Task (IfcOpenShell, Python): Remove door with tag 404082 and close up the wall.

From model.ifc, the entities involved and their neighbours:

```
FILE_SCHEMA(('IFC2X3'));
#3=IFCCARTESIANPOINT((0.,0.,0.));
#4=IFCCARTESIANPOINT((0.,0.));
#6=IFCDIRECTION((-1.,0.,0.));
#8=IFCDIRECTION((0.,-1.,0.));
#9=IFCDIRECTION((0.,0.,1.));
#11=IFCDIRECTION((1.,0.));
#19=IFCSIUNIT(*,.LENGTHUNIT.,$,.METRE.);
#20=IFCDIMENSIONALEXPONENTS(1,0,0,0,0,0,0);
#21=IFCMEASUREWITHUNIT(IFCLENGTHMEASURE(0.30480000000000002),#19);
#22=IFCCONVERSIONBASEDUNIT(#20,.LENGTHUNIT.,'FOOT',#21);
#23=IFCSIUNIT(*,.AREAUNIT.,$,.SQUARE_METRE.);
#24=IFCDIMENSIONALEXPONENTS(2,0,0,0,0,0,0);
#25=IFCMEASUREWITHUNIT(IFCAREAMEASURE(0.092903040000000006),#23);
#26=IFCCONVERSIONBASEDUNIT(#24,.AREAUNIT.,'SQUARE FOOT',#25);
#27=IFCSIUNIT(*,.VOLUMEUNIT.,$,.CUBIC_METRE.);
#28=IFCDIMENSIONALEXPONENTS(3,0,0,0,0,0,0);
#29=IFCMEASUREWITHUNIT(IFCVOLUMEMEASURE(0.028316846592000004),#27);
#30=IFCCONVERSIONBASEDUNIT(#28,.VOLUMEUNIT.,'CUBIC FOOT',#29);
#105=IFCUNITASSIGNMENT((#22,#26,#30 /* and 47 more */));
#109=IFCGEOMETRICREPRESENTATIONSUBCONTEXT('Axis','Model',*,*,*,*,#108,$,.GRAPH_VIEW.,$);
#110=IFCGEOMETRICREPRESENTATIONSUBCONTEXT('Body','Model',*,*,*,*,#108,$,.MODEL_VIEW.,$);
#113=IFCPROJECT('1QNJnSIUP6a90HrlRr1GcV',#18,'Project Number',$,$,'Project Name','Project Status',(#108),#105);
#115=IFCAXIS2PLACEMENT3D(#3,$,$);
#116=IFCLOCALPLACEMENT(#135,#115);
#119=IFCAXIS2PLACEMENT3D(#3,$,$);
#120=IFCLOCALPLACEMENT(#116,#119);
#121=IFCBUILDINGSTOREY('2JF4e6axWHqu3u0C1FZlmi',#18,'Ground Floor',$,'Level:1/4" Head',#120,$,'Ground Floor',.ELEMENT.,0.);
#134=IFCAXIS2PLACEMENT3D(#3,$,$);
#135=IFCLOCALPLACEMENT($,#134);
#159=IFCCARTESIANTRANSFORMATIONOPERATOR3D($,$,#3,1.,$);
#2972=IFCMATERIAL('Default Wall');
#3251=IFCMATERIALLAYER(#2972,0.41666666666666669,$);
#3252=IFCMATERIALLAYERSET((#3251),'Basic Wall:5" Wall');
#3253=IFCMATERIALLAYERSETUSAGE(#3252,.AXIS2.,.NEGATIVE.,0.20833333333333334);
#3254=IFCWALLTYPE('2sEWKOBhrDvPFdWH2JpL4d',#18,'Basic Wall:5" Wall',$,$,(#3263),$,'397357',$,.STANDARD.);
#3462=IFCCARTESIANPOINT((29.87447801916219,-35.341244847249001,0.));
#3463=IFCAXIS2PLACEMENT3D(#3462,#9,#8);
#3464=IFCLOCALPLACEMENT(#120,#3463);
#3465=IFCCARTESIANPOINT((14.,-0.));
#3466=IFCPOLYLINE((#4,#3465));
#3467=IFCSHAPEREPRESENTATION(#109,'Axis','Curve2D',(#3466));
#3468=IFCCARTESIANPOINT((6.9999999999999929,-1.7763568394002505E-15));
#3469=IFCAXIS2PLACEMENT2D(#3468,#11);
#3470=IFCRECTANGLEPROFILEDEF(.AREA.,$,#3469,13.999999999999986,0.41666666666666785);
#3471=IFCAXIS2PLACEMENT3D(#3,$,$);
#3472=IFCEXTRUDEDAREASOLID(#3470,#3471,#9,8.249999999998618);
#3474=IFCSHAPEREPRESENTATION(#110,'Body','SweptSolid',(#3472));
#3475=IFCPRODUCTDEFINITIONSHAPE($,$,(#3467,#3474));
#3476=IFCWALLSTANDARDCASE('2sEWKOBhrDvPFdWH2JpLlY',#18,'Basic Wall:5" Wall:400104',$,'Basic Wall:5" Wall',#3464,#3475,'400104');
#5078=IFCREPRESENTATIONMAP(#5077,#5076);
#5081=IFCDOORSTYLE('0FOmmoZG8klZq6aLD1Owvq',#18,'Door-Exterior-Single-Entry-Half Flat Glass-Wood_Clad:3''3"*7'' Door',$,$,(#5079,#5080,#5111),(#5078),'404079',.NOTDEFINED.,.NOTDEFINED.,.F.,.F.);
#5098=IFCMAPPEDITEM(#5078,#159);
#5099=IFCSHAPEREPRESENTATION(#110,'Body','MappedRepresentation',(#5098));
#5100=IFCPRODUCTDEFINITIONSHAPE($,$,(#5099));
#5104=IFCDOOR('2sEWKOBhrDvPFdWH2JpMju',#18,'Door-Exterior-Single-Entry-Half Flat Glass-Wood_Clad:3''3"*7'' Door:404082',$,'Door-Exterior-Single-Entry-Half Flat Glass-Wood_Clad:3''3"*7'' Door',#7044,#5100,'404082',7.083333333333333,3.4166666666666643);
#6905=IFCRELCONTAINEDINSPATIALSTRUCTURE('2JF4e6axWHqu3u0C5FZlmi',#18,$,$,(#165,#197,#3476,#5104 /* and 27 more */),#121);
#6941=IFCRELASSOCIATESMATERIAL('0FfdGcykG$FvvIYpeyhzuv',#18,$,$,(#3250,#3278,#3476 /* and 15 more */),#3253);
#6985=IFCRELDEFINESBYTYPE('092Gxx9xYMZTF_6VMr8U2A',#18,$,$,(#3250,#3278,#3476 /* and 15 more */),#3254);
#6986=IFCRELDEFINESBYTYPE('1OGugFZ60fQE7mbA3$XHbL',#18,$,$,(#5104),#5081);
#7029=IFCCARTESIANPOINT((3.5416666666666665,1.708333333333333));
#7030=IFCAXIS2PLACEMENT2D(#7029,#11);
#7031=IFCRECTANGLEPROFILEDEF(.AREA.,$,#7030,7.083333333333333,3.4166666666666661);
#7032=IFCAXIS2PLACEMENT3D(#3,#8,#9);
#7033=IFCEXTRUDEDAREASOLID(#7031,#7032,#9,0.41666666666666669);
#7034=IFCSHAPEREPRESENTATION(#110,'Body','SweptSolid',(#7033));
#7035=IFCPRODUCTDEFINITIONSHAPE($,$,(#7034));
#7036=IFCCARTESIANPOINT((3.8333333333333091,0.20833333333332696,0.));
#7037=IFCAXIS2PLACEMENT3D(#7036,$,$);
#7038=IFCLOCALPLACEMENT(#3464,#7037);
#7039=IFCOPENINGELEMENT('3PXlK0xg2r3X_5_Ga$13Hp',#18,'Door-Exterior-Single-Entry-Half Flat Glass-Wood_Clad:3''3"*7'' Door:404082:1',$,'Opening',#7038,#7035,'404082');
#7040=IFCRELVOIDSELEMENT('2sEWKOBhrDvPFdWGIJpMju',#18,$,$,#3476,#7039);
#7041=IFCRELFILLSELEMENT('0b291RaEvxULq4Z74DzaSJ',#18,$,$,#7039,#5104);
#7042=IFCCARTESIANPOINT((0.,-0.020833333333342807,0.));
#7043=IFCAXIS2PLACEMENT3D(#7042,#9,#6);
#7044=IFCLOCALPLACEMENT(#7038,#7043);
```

```python
import ifcopenshell
import ifcopenshell.api.feature
import ifcopenshell.api.root
import ifcopenshell.geom
import ifcopenshell.util.shape

model = ifcopenshell.open("model.ifc")
settings = ifcopenshell.geom.settings()


def volume(element):
    """Net volume in cubic metres, openings subtracted."""
    shape = ifcopenshell.geom.create_shape(settings, element)
    return ifcopenshell.util.shape.get_volume(shape.geometry)


door = model.by_id(5104)
opening = door.FillsVoids[0].RelatingOpeningElement
wall = opening.VoidsElements[0].RelatingBuildingElement
before = volume(wall)

ifcopenshell.api.root.remove_product(model, product=door)
ifcopenshell.api.feature.remove_feature(model, feature=opening)

after = volume(wall)

print(f"wall volume {before:.3f} -> {after:.3f} m3")

model.write("model_v2.ifc")
```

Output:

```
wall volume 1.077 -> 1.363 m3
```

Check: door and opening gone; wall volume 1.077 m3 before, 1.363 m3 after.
